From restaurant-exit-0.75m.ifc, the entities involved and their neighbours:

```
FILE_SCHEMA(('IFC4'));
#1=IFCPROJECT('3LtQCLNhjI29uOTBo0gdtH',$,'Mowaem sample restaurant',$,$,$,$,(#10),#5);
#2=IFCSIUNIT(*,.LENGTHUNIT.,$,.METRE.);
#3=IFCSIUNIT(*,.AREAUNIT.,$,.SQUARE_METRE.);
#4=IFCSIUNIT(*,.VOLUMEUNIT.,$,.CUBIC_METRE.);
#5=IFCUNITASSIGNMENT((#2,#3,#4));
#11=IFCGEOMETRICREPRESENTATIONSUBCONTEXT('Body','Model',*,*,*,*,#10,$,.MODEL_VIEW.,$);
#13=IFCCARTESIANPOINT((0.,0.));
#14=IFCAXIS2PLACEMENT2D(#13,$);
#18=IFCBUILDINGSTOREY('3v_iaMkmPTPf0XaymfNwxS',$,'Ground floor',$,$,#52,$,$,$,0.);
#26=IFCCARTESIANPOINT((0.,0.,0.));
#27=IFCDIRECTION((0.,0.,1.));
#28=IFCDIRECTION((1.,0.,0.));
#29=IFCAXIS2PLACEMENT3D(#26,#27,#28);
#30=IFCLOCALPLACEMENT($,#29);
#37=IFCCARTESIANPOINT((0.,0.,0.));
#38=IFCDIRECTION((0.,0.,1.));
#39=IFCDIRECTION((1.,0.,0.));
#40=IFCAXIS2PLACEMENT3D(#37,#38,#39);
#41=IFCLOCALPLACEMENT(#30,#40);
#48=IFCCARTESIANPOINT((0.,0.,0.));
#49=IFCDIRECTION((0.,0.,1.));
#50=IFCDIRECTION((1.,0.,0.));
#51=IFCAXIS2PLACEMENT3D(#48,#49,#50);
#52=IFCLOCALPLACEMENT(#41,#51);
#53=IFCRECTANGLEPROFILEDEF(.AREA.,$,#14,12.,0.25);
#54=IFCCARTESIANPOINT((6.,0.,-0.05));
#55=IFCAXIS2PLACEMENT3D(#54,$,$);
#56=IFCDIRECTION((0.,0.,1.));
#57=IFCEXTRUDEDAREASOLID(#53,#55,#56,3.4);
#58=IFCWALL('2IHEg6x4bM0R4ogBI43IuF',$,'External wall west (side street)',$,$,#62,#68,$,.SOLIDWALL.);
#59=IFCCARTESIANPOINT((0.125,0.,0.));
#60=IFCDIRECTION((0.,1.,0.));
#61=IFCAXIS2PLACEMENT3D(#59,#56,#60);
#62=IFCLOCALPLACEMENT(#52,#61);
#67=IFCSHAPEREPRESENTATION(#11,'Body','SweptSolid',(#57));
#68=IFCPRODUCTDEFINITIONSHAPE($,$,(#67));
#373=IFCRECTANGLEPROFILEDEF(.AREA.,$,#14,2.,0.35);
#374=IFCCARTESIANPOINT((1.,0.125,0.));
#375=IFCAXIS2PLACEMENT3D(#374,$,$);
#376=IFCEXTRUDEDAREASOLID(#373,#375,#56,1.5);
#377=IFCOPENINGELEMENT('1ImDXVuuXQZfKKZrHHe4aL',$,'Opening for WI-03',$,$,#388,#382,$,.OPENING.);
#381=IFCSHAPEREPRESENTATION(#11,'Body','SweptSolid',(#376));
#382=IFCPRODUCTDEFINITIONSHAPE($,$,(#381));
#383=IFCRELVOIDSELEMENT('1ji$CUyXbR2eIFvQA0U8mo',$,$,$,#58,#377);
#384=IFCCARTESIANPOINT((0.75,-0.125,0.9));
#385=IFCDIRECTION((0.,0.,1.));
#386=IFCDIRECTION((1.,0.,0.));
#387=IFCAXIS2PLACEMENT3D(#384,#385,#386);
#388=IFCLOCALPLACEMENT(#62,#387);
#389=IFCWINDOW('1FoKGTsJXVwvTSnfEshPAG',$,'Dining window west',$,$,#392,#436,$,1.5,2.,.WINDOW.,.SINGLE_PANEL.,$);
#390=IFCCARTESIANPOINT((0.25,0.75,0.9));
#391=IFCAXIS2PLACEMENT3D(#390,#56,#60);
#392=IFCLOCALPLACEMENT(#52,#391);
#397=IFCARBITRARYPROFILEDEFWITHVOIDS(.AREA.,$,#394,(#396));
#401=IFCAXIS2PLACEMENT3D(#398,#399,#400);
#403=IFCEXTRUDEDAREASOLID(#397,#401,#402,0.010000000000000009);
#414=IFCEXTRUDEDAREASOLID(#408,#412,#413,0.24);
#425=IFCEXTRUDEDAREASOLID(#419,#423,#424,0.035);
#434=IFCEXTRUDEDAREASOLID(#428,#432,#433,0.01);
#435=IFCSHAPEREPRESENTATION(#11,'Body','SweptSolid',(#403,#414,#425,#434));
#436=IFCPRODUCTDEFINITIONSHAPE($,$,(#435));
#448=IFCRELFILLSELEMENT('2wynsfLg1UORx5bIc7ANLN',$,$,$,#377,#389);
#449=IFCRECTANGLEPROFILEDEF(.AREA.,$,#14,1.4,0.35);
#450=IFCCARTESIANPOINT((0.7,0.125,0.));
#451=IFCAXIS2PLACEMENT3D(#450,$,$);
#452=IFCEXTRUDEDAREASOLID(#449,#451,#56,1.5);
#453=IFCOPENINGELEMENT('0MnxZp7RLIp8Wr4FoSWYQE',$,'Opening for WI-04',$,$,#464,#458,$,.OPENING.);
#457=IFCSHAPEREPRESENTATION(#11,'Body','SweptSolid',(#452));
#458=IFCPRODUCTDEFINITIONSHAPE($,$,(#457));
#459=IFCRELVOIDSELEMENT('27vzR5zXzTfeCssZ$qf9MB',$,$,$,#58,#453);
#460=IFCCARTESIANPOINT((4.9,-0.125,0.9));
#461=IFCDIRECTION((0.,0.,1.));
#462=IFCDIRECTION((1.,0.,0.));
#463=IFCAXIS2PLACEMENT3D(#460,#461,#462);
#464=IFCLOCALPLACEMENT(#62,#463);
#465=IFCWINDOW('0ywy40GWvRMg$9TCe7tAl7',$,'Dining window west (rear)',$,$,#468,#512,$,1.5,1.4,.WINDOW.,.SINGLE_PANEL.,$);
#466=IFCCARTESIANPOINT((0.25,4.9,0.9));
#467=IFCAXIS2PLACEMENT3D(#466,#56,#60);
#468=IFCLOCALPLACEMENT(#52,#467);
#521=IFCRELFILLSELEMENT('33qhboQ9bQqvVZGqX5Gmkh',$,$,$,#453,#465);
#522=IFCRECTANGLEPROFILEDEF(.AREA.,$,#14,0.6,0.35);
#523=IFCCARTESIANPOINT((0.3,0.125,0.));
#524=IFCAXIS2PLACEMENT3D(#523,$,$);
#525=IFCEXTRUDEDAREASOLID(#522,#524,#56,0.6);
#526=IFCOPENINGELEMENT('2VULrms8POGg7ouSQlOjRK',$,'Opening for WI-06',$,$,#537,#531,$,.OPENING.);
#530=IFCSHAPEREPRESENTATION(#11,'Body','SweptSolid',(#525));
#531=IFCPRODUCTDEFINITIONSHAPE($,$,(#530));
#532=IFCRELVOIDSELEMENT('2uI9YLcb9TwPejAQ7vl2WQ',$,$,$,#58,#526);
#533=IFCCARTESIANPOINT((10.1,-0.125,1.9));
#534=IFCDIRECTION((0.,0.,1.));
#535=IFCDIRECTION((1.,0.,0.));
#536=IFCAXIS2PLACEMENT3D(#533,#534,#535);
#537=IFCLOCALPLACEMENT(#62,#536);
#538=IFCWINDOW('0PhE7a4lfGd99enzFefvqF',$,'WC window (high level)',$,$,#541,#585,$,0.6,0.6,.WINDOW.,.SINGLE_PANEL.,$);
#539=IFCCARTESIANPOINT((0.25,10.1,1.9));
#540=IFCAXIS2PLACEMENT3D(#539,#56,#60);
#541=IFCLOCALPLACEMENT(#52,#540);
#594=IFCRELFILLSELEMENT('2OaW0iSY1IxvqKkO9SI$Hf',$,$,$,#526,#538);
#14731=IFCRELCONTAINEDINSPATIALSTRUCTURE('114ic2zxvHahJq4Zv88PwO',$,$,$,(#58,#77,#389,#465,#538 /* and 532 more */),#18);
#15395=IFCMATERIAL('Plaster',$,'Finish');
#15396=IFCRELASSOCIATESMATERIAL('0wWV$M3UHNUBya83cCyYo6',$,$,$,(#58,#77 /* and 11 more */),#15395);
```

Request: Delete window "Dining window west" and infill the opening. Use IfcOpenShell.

```python
import ifcopenshell
import ifcopenshell.api.feature
import ifcopenshell.api.root
import ifcopenshell.geom
import ifcopenshell.util.shape

model = ifcopenshell.open("restaurant-exit-0.75m.ifc")
settings = ifcopenshell.geom.settings()


def volume(element):
    """Net volume in cubic metres, openings subtracted."""
    shape = ifcopenshell.geom.create_shape(settings, element)
    return ifcopenshell.util.shape.get_volume(shape.geometry)


window = model.by_id(389)
opening = window.FillsVoids[0].RelatingOpeningElement
wall = opening.VoidsElements[0].RelatingBuildingElement
before = volume(wall)

ifcopenshell.api.root.remove_product(model, product=window)
ifcopenshell.api.feature.remove_feature(model, feature=opening)

after = volume(wall)

print(f"wall volume {before:.3f} -> {after:.3f} m3")

model.write("restaurant-exit-0.75m_rev.ifc")
```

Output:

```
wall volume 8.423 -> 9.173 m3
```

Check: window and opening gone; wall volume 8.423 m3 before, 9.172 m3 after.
